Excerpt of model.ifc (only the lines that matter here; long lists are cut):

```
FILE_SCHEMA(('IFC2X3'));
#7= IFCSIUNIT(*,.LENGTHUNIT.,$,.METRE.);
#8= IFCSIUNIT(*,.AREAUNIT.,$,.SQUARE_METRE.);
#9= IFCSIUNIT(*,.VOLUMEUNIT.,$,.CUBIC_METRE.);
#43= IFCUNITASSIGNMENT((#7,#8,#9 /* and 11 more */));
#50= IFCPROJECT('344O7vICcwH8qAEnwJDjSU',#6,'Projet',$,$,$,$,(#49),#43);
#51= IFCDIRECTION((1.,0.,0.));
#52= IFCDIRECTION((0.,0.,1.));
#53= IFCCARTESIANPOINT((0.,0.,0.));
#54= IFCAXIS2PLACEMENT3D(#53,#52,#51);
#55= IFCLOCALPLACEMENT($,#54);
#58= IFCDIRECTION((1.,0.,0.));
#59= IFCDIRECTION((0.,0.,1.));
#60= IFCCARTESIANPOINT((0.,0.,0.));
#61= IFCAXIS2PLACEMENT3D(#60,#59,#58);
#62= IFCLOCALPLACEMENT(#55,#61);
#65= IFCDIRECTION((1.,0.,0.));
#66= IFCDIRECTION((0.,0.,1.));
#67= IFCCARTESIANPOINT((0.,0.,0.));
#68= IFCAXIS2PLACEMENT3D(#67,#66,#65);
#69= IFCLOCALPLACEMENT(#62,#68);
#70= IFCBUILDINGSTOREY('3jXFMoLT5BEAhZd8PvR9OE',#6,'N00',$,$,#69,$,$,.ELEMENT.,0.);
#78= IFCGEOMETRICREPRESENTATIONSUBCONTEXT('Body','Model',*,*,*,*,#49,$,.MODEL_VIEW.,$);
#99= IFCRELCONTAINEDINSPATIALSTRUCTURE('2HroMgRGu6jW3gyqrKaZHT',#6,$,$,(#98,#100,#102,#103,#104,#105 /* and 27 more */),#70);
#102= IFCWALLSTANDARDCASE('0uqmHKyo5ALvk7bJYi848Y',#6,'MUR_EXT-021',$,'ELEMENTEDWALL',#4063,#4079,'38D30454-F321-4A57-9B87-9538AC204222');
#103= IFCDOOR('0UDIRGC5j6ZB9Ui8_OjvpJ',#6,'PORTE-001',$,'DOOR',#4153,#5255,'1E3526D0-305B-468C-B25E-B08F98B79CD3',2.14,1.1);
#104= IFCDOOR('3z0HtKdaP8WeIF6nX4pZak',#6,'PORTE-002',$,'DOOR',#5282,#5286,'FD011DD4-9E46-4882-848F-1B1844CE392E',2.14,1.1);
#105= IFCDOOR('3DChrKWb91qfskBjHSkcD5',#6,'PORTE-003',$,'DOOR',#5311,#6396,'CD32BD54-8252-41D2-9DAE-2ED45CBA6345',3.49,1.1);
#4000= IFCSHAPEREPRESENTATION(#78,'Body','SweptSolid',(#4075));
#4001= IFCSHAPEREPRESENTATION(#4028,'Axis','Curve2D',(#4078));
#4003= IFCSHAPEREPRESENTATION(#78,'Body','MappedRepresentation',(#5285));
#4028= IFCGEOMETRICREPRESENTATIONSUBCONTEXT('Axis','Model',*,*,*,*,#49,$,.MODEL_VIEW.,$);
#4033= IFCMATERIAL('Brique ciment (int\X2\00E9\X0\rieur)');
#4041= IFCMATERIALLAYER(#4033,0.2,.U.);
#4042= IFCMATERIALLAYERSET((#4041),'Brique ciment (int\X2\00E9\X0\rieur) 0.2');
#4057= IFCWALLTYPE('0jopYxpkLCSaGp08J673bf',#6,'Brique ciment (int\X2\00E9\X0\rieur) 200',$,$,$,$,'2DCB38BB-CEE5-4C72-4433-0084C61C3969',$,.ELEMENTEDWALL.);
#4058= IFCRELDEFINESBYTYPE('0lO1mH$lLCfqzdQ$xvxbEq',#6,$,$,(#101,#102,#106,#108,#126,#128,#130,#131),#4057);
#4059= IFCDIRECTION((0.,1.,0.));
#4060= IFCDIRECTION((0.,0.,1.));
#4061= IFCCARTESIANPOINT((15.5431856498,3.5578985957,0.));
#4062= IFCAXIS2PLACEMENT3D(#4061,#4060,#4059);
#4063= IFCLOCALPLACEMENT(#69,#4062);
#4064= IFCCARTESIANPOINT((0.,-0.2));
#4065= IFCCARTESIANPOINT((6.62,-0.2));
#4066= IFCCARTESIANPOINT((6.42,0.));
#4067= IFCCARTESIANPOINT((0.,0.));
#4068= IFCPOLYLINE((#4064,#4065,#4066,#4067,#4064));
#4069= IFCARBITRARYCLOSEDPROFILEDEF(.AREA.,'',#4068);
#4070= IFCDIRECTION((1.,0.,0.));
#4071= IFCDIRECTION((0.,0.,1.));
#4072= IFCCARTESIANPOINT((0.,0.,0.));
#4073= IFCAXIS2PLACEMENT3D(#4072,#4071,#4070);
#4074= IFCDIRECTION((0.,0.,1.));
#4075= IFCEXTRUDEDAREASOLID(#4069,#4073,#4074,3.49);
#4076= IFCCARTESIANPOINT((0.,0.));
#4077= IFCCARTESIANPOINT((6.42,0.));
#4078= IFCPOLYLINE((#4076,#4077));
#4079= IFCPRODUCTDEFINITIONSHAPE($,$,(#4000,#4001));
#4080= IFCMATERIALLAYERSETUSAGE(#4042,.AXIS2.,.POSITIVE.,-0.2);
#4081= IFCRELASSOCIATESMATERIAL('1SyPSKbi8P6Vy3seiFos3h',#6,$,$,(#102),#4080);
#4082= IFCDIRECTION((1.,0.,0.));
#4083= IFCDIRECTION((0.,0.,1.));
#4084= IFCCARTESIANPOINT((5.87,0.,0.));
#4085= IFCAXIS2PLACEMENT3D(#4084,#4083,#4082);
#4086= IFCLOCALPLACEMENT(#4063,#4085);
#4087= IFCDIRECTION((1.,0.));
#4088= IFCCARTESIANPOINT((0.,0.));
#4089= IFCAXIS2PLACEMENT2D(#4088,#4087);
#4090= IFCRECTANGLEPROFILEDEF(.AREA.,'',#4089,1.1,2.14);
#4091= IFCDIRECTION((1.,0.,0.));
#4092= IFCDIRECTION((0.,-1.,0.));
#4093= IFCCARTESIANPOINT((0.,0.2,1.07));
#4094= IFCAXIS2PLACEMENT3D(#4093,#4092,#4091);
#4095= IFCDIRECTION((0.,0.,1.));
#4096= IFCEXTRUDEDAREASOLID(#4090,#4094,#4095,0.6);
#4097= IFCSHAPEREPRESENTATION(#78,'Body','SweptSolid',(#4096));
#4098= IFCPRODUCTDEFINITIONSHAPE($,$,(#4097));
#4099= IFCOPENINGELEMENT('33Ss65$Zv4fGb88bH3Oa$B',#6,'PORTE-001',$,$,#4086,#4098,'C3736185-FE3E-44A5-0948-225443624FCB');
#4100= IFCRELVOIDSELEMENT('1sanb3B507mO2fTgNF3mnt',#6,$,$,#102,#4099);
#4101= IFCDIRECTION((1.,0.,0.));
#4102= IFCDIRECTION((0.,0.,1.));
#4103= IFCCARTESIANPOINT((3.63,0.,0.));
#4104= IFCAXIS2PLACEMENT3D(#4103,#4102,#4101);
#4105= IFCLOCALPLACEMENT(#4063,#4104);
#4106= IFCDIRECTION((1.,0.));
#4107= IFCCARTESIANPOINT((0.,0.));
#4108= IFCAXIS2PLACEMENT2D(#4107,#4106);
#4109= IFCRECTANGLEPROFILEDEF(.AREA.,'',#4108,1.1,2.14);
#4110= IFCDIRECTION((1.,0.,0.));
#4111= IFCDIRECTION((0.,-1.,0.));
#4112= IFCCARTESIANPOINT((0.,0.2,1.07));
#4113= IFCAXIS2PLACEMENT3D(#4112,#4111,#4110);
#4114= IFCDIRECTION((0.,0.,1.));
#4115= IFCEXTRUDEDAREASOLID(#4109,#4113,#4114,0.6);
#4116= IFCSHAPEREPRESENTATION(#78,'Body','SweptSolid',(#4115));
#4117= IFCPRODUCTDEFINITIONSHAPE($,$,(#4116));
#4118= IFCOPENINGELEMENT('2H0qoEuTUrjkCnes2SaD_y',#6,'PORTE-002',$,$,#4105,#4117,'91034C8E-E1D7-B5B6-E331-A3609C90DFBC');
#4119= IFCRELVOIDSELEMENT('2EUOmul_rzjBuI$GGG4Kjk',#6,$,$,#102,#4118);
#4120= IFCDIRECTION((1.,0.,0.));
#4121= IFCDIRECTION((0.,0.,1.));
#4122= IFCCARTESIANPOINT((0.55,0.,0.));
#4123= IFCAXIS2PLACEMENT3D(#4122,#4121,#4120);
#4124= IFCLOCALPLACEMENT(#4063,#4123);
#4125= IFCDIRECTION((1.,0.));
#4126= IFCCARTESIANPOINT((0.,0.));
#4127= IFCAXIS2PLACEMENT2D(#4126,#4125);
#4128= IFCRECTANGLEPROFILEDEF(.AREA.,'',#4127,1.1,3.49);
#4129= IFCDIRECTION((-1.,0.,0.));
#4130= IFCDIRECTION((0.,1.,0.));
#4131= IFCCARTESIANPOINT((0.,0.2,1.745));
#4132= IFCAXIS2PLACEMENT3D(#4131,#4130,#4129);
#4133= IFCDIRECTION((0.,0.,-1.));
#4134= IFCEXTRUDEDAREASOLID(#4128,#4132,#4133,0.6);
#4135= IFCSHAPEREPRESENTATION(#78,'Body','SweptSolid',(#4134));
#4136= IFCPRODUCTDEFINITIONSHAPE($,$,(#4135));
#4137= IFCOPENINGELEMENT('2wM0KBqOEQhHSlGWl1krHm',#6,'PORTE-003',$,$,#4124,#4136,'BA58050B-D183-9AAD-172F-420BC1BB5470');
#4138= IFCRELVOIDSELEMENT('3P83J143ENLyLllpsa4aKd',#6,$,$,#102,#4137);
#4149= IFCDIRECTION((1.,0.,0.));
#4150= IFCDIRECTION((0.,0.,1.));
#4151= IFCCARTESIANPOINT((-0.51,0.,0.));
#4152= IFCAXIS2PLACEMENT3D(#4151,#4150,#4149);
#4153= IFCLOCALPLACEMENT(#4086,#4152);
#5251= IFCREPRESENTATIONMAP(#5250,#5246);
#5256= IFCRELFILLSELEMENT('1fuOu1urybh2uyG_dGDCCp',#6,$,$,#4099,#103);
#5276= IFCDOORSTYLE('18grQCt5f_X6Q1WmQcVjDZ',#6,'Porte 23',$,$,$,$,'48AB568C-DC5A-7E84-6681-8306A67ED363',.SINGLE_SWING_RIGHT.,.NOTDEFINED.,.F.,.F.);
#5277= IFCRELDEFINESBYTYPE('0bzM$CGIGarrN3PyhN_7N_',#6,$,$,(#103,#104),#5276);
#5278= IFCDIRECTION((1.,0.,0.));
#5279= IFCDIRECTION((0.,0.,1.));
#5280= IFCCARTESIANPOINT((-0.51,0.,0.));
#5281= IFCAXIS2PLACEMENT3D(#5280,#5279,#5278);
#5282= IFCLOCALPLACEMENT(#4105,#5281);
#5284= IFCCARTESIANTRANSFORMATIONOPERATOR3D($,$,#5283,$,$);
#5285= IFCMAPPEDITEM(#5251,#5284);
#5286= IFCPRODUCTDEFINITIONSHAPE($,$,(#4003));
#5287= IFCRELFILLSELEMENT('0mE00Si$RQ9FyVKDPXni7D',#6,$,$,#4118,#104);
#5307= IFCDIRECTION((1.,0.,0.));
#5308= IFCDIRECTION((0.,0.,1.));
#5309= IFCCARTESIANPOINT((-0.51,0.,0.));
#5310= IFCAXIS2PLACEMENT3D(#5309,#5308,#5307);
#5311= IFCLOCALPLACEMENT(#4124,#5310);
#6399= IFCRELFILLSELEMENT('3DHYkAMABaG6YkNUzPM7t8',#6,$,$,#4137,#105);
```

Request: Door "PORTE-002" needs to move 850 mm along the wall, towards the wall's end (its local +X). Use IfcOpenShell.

```python
import ifcopenshell
import ifcopenshell.api.geometry
import ifcopenshell.util.placement
import ifcopenshell.util.unit

model = ifcopenshell.open("model.ifc")
unit_scale = ifcopenshell.util.unit.calculate_unit_scale(model)

door = model.by_guid("3z0HtKdaP8WeIF6nX4pZak")
opening = door.FillsVoids[0].RelatingOpeningElement
wall = opening.VoidsElements[0].RelatingBuildingElement

wall_matrix = ifcopenshell.util.placement.get_local_placement(wall.ObjectPlacement)
shift = wall_matrix[:3, 0] * 0.85 / unit_scale
before = ifcopenshell.util.placement.get_local_placement(door.ObjectPlacement)[:3, 3].copy()

# The door is placed relative to its opening, so it follows when the opening moves.
matrix = ifcopenshell.util.placement.get_local_placement(opening.ObjectPlacement)
matrix[:3, 3] += shift
ifcopenshell.api.geometry.edit_object_placement(
    model, product=opening, matrix=matrix, is_si=False, should_transform_children=True
)

after = ifcopenshell.util.placement.get_local_placement(door.ObjectPlacement)[:3, 3]
print("door moved by", (after - before).round(3) + 0.0)

model.write("model_v2.ifc")
```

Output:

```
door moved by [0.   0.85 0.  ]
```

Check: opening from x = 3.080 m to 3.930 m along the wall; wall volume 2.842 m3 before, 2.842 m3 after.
